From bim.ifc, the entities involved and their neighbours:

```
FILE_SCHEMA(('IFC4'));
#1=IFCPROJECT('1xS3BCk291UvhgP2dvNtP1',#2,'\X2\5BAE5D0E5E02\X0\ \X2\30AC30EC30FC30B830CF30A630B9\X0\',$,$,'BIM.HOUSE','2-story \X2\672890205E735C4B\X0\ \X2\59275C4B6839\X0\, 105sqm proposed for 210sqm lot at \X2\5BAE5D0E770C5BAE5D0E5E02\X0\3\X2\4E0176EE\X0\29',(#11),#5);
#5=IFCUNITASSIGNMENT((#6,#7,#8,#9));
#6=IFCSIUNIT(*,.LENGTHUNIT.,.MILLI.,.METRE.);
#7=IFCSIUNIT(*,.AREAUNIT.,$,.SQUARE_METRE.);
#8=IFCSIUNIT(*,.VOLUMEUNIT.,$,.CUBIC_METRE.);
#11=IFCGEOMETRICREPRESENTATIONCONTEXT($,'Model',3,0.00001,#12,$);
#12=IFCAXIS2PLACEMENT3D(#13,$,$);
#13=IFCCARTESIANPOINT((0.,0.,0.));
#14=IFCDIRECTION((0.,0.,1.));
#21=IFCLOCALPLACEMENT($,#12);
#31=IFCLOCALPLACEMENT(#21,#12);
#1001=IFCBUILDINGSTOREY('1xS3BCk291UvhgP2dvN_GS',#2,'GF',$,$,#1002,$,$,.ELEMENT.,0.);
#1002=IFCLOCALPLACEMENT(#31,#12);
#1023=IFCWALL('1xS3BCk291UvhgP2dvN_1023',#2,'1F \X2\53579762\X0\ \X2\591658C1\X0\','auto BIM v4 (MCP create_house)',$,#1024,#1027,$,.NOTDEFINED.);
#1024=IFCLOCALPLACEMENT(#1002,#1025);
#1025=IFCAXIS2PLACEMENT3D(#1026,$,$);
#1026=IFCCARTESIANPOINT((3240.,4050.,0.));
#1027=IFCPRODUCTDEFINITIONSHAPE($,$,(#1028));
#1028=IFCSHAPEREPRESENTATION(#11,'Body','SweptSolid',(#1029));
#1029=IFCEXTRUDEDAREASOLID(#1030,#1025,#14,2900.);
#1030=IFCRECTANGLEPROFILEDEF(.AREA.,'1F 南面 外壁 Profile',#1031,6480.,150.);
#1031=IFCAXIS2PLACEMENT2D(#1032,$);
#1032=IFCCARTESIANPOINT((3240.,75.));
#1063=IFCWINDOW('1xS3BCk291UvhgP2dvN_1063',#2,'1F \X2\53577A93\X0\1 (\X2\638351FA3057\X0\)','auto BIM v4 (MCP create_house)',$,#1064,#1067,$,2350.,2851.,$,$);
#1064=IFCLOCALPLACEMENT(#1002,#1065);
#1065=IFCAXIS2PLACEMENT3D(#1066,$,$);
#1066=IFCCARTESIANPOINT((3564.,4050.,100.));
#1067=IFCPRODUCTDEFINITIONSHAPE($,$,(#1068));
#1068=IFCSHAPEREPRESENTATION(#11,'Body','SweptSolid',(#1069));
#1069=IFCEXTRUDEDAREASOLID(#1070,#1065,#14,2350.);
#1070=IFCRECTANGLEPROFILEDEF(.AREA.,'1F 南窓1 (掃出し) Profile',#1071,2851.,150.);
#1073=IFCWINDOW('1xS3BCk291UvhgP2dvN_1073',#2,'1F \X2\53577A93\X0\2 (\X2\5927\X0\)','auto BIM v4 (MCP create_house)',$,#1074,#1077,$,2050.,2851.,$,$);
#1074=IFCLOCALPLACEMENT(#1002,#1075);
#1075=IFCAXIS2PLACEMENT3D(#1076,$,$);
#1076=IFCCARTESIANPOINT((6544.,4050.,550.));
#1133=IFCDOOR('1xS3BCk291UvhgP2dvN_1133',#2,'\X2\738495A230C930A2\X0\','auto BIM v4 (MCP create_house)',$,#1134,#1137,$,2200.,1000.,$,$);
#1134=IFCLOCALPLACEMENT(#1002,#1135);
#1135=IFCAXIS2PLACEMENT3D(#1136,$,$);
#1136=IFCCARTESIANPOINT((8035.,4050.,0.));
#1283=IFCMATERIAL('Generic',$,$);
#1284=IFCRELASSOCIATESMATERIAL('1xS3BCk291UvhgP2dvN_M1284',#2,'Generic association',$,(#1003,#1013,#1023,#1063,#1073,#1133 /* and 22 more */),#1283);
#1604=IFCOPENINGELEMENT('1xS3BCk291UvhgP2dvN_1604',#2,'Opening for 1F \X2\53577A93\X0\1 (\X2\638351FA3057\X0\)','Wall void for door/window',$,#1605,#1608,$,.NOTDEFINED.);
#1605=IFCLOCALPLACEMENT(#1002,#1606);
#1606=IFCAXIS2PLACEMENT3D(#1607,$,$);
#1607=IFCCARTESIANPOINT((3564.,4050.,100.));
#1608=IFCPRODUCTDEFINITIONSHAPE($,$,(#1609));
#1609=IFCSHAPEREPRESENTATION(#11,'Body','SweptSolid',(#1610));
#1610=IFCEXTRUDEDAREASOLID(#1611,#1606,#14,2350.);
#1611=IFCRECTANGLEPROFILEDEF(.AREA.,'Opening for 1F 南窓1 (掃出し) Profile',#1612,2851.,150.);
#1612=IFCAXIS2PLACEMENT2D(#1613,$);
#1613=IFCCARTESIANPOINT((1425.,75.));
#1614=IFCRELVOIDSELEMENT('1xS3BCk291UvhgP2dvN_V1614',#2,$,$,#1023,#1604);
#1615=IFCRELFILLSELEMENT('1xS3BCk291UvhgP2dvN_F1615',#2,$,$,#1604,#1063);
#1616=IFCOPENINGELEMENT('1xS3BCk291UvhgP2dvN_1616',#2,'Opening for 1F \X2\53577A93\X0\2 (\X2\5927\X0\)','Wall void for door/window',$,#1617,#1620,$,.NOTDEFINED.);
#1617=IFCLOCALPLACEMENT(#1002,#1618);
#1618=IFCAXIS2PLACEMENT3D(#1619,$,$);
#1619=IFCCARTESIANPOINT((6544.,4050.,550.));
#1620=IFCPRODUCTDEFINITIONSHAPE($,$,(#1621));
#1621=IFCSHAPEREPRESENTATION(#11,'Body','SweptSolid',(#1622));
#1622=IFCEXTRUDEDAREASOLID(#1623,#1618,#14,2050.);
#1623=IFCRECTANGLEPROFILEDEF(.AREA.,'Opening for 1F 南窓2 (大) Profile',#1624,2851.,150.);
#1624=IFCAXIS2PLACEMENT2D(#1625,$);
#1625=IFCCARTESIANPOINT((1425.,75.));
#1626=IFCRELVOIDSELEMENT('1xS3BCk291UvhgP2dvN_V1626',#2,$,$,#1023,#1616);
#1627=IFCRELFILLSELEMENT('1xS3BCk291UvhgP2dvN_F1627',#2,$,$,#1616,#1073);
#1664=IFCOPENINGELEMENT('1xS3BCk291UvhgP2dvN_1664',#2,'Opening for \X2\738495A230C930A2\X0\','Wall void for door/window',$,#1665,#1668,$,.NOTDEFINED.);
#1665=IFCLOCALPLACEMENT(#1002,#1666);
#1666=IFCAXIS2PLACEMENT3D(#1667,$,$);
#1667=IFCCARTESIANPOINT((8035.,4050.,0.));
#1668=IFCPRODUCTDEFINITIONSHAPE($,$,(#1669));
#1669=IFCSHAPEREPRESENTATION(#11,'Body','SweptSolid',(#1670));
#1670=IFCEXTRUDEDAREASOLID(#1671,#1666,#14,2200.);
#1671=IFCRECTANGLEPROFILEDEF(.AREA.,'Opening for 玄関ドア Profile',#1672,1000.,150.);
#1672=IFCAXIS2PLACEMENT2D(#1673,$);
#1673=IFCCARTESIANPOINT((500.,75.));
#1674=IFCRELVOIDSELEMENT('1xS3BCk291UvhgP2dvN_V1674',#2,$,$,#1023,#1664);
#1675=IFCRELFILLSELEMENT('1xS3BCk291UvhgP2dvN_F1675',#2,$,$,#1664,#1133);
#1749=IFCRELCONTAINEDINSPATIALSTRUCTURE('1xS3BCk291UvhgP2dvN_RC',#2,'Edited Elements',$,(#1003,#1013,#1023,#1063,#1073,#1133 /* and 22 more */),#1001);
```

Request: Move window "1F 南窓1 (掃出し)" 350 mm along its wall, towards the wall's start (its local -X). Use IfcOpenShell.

```python
import ifcopenshell
import ifcopenshell.api.geometry
import ifcopenshell.util.placement

model = ifcopenshell.open("bim.ifc")

window = model.by_guid("1xS3BCk291UvhgP2dvN_1063")
opening = window.FillsVoids[0].RelatingOpeningElement
wall = opening.VoidsElements[0].RelatingBuildingElement

wall_matrix = ifcopenshell.util.placement.get_local_placement(wall.ObjectPlacement)
shift = wall_matrix[:3, 0] * -350.0
before = ifcopenshell.util.placement.get_local_placement(window.ObjectPlacement)[:3, 3].copy()

# The window is not placed relative to its opening, so move both.
for product in (opening, window):
    matrix = ifcopenshell.util.placement.get_local_placement(product.ObjectPlacement)
    matrix[:3, 3] += shift
    ifcopenshell.api.geometry.edit_object_placement(model, product=product, matrix=matrix, is_si=False)

after = ifcopenshell.util.placement.get_local_placement(window.ObjectPlacement)[:3, 3]
print("window moved by", (after - before).round(3) + 0.0)

model.write("bim_edited.ifc")
```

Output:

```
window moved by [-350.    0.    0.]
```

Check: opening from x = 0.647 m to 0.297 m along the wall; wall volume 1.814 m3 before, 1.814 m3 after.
